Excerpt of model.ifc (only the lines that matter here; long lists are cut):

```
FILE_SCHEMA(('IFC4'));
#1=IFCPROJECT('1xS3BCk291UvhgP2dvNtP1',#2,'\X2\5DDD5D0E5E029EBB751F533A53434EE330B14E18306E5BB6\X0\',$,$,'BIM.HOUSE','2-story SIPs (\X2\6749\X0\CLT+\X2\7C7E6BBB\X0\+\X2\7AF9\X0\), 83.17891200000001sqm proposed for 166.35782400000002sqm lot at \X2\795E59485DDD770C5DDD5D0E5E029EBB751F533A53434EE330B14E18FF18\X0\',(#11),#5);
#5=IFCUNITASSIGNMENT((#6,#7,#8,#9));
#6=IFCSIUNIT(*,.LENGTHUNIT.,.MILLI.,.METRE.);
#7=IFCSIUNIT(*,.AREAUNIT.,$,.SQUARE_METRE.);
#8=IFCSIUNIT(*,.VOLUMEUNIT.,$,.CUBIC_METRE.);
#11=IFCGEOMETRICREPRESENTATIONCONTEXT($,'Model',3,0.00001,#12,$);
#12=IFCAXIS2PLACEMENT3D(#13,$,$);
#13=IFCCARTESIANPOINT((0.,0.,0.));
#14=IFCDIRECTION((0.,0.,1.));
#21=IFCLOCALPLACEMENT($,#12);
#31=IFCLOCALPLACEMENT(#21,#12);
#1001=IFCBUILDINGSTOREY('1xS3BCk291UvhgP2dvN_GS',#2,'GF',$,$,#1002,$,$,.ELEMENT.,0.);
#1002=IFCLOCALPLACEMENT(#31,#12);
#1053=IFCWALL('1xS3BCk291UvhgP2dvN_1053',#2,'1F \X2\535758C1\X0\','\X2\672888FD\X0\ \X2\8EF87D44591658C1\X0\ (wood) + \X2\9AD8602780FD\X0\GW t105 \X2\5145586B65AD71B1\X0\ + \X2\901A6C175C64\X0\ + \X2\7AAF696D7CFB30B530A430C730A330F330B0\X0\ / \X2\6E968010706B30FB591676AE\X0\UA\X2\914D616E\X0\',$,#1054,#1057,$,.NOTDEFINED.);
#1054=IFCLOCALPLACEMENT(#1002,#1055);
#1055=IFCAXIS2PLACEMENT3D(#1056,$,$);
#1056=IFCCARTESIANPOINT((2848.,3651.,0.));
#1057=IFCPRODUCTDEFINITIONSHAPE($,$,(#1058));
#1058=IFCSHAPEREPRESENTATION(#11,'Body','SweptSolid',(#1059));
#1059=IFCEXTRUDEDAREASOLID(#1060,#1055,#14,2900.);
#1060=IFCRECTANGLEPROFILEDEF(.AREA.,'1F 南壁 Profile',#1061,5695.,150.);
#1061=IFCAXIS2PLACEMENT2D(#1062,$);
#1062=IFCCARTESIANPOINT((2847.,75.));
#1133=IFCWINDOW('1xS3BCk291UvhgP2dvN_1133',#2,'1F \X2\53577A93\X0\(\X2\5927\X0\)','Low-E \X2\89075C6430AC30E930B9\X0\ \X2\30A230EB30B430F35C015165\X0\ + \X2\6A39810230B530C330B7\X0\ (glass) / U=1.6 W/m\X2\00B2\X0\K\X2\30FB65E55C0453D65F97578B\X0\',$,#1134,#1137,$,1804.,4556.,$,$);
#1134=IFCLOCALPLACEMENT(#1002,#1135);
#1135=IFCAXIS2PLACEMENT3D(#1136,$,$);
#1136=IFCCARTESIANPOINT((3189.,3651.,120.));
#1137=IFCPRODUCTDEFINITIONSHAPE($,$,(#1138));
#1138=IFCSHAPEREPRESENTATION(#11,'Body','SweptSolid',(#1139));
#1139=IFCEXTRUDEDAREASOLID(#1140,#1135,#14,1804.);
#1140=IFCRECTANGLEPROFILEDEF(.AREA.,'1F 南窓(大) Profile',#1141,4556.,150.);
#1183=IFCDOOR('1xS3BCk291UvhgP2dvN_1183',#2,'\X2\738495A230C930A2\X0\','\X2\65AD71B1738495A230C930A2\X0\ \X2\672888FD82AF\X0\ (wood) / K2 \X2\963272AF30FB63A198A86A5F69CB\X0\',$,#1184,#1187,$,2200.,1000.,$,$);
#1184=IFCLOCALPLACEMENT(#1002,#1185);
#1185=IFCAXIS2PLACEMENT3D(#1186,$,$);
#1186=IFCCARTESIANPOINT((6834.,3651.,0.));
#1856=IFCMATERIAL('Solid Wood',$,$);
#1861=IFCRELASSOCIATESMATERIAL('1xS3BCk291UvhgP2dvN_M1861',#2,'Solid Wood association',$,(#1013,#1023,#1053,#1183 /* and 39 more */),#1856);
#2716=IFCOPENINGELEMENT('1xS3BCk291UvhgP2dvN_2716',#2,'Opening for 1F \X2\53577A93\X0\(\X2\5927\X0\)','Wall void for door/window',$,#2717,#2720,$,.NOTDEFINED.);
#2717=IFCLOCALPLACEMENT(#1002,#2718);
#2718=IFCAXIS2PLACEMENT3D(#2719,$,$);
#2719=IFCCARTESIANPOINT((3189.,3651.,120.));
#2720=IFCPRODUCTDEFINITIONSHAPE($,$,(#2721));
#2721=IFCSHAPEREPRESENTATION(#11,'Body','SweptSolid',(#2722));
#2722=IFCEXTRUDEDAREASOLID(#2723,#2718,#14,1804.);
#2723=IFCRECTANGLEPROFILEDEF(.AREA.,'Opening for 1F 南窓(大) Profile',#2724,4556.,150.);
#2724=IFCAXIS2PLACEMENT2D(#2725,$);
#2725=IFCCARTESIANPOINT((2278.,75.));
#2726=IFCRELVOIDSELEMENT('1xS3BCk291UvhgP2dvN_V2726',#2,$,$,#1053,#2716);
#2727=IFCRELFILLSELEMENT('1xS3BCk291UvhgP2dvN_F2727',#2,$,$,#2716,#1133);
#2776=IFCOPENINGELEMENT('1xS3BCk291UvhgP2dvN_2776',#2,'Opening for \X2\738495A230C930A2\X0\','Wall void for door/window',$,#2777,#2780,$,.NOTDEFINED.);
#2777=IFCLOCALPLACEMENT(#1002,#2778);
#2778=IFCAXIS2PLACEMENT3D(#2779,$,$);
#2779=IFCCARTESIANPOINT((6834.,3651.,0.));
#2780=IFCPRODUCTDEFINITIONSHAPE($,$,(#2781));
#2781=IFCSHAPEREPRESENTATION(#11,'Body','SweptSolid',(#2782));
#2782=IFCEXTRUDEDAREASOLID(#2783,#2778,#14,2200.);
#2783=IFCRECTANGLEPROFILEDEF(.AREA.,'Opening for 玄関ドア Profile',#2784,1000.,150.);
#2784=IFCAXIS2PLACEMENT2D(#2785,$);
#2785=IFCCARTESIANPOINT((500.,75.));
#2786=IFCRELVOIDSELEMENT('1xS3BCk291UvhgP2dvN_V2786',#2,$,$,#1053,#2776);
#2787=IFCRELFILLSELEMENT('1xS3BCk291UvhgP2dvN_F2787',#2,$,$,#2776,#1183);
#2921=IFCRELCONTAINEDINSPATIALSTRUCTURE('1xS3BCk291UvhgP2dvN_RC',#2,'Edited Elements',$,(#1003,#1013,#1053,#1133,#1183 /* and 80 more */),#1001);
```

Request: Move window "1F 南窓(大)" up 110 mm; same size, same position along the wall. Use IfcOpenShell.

```python
import numpy as np
import ifcopenshell
import ifcopenshell.api.geometry
import ifcopenshell.util.placement
import ifcopenshell.util.unit

model = ifcopenshell.open("model.ifc")
unit_scale = ifcopenshell.util.unit.calculate_unit_scale(model)

window = model.by_id(1133)
opening = window.FillsVoids[0].RelatingOpeningElement
dz = 0.11 / unit_scale

shift = np.array([0.0, 0.0, dz])
# The window is not placed relative to its opening, so move both.
for product in (opening, window):
    matrix = ifcopenshell.util.placement.get_local_placement(product.ObjectPlacement)
    matrix[:3, 3] += shift
    ifcopenshell.api.geometry.edit_object_placement(model, product=product, matrix=matrix, is_si=False)

print(f"moved by {dz * unit_scale:+.3f} m")

model.write("model_v2.ifc")
```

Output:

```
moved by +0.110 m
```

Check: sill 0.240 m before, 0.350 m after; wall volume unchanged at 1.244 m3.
